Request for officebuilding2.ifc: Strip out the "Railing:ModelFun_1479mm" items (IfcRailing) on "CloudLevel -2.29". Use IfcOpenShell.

First a look at what the model holds.

```python
import ifcopenshell
import ifcopenshell.util.element

model = ifcopenshell.open("officebuilding2.ifc")
print(model.schema)
storey = next(s for s in model.by_type("IfcBuildingStorey") if s.Name == "CloudLevel -2.29")
railings = [e for e in ifcopenshell.util.element.get_decomposition(storey) if e.is_a("IfcRailing")]
seen = {}
for e in railings:
    element_type = ifcopenshell.util.element.get_type(e)
    name = element_type.Name if element_type not in (None, e) else None
    seen[name] = seen.get(name, 0) + 1
for name, count in sorted(seen.items(), key=str):
    print(count, "x", name)
```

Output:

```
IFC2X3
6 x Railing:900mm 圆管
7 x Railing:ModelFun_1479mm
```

```python
import ifcopenshell
import ifcopenshell.api.root
import ifcopenshell.util.element

model = ifcopenshell.open("officebuilding2.ifc")

storey = next(s for s in model.by_type("IfcBuildingStorey") if s.Name == "CloudLevel -2.29")
railings = [e for e in ifcopenshell.util.element.get_decomposition(storey) if e.is_a("IfcRailing")]
targets = [e for e in railings if (t := ifcopenshell.util.element.get_type(e)) not in (None, e) and t.Name == "Railing:ModelFun_1479mm"]

for e in targets:
    ifcopenshell.api.root.remove_product(model, product=e)
print(len(targets), "removed")

model.write("officebuilding2_rev.ifc")
```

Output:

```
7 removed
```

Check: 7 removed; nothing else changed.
